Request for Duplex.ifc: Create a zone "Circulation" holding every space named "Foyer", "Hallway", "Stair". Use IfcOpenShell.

First a look at what the model holds.

```python
import ifcopenshell

model = ifcopenshell.open("Duplex.ifc")
print(model.schema)
seen = {}
for space in model.by_type("IfcSpace"):
    seen[space.LongName] = seen.get(space.LongName, 0) + 1
for name, count in sorted(seen.items(), key=str):
    print(count, "x", name)
print("zones:", [z.Name for z in model.by_type("IfcZone")][:20])
```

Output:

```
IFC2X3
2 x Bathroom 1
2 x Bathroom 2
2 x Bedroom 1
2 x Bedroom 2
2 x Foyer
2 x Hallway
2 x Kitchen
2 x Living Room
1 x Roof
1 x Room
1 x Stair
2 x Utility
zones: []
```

```python
import ifcopenshell
import ifcopenshell.api.group
import ifcopenshell.api.root

model = ifcopenshell.open("Duplex.ifc")

names = {"Foyer", "Hallway", "Stair"}
spaces = [s for s in model.by_type("IfcSpace") if s.LongName in names]

zone = ifcopenshell.api.root.create_entity(model, ifc_class="IfcZone", name="Circulation")
ifcopenshell.api.group.assign_group(model, products=spaces, group=zone)
print(len(spaces), "spaces in", zone.Name)

model.write("Duplex_edited.ifc")
```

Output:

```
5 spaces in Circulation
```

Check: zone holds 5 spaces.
